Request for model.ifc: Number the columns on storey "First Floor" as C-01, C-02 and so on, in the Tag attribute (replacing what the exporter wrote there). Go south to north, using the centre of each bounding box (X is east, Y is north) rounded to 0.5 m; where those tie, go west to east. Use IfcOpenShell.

First a look at what the model holds.

```python
import ifcopenshell
import ifcopenshell.util.element
import ifcopenshell.util.placement

model = ifcopenshell.open("model.ifc")
print(model.schema)
storey = next(s for s in model.by_type("IfcBuildingStorey") if s.Name == "First Floor")
columns = [e for e in ifcopenshell.util.element.get_decomposition(storey) if e.is_a("IfcColumn")]
for e in sorted(columns, key=lambda e: e.id()):
    origin = ifcopenshell.util.placement.get_local_placement(e.ObjectPlacement)[:3, 3]
    print(e.id(), e.Tag, e.Name, origin.round(2) + 0.0, sep=" | ")
```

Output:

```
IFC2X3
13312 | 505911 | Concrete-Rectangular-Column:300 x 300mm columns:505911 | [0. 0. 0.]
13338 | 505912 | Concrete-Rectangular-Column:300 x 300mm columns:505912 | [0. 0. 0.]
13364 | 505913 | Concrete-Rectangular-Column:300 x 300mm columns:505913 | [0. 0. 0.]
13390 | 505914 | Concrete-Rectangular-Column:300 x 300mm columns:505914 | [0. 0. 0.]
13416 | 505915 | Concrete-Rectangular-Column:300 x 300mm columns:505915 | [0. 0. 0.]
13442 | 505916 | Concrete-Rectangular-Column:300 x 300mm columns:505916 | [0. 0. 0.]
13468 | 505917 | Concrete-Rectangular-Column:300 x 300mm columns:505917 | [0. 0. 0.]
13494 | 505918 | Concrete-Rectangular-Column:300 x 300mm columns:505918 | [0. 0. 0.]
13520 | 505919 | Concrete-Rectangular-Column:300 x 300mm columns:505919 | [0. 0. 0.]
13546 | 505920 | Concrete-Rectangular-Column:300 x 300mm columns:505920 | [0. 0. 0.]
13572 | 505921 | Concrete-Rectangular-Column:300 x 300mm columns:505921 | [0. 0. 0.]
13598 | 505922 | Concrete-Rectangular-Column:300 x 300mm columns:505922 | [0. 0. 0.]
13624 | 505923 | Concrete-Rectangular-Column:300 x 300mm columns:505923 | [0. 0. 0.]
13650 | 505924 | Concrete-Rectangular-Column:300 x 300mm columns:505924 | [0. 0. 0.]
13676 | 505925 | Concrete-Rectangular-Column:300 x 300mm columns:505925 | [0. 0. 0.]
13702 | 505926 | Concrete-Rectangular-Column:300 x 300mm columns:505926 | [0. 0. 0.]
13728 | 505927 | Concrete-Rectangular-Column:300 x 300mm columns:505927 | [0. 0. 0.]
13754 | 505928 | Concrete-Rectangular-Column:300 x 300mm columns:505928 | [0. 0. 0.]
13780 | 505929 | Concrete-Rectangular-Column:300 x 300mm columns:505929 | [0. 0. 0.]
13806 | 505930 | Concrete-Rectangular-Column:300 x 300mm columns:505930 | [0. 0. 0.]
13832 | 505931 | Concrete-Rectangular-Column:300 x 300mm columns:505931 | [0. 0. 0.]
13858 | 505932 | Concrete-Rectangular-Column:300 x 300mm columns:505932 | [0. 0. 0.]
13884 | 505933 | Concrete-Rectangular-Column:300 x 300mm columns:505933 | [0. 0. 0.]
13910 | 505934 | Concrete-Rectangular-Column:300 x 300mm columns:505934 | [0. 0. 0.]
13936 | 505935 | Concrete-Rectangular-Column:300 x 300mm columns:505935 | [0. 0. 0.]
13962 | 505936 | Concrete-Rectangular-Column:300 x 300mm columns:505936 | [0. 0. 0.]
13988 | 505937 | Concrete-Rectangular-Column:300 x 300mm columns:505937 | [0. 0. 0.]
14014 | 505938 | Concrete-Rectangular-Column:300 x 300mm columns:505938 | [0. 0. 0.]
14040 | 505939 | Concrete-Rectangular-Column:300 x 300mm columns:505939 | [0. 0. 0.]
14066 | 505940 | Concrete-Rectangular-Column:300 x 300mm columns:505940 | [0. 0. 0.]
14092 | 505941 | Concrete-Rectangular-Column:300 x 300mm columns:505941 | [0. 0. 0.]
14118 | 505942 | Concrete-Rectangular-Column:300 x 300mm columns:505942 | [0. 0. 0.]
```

```python
import ifcopenshell
import ifcopenshell.geom
import ifcopenshell.util.element
import ifcopenshell.util.shape

model = ifcopenshell.open("model.ifc")
settings = ifcopenshell.geom.settings()
settings.set("use-world-coords", True)


def centre(element):
    shape = ifcopenshell.geom.create_shape(settings, element)
    return ifcopenshell.util.shape.get_bbox_centroid(shape.geometry)


storey = next(s for s in model.by_type("IfcBuildingStorey") if s.Name == "First Floor")
columns = [e for e in ifcopenshell.util.element.get_decomposition(storey) if e.is_a("IfcColumn")]

# Insertion points can sit at a corner or the storey origin, so sort by the geometry (in metres).
centres = {e: centre(e) for e in columns}
columns.sort(key=lambda e: (round(centres[e][1] / 0.5), centres[e][0]))

for i, e in enumerate(columns, start=1):
    number = f"C-{i:02d}"
    e.Tag = number
    print(e.id(), number)

model.write("model_v2.ifc")
```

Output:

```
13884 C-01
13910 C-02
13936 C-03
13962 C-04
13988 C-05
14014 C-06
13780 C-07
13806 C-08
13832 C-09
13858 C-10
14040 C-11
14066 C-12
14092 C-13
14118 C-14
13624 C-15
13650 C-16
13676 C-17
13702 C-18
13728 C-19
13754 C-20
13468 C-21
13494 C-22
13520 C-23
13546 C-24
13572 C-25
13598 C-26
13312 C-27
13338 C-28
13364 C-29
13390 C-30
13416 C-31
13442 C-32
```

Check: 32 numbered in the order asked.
